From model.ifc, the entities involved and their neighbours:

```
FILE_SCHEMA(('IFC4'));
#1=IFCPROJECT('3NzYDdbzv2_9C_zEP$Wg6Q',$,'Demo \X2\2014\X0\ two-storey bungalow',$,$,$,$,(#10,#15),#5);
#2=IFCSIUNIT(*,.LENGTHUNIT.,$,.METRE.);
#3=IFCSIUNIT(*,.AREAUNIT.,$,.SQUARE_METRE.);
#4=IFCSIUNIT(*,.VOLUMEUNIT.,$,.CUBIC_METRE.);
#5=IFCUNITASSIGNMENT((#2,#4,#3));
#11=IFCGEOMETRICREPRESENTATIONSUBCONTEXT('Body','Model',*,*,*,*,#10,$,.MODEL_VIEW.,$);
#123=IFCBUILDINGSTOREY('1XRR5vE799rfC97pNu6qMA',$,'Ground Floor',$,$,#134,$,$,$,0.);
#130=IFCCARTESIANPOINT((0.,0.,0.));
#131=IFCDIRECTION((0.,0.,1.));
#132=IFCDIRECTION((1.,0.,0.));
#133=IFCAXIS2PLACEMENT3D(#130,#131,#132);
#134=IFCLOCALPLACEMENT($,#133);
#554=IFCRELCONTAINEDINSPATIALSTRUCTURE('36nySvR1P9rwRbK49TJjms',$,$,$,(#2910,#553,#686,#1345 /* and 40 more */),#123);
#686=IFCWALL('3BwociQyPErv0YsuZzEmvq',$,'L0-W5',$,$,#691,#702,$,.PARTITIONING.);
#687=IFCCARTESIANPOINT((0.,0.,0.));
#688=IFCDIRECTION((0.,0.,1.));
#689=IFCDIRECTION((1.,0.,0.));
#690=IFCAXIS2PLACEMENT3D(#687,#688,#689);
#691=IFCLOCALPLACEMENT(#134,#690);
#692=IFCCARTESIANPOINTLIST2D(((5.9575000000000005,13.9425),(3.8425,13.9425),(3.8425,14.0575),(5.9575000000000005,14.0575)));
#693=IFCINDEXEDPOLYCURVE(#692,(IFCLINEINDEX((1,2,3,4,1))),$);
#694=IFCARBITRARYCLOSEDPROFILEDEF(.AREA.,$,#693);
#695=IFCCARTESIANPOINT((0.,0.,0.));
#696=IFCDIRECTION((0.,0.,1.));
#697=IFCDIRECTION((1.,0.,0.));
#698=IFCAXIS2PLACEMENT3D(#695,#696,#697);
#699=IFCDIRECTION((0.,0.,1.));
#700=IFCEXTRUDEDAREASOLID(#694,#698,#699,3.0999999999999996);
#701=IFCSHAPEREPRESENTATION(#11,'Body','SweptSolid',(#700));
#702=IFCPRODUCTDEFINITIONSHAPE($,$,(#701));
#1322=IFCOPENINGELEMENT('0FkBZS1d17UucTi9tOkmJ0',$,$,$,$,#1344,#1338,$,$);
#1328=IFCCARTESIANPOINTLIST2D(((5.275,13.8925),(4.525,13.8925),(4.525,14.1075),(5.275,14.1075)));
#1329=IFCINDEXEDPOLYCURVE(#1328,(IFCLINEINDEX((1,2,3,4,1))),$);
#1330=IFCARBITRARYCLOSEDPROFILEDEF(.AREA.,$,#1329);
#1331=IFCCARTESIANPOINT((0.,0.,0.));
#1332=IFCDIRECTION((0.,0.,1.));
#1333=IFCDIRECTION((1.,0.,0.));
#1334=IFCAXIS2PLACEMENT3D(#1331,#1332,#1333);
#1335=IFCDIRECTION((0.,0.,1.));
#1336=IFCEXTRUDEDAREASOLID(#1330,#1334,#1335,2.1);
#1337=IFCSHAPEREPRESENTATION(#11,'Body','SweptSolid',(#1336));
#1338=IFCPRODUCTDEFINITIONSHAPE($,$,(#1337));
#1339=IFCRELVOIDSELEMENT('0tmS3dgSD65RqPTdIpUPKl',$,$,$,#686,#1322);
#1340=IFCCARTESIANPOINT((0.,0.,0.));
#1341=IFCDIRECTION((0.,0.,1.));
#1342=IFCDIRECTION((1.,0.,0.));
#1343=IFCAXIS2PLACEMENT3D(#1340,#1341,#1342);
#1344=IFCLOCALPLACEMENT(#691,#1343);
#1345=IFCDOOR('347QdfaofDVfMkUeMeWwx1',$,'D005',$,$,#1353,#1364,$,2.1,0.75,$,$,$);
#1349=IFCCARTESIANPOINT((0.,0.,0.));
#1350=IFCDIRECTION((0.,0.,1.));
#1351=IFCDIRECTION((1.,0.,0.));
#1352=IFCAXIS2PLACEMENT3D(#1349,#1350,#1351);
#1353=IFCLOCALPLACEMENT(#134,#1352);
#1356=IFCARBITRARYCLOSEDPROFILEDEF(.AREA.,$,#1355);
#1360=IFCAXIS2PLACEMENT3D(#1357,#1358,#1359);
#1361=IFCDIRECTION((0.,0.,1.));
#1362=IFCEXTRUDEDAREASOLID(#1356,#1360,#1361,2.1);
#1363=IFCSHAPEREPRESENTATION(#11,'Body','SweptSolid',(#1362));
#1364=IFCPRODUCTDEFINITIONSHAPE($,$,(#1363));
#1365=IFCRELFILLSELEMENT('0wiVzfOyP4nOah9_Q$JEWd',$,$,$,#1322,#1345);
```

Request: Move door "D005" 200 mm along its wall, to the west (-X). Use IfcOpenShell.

```python
import ifcopenshell
import ifcopenshell.api.geometry
import ifcopenshell.util.placement
import ifcopenshell.util.unit

model = ifcopenshell.open("model.ifc")
unit_scale = ifcopenshell.util.unit.calculate_unit_scale(model)

door = model.by_guid("347QdfaofDVfMkUeMeWwx1")
opening = door.FillsVoids[0].RelatingOpeningElement
wall = opening.VoidsElements[0].RelatingBuildingElement

wall_matrix = ifcopenshell.util.placement.get_local_placement(wall.ObjectPlacement)
shift = wall_matrix[:3, 0] * -0.2 / unit_scale
before = ifcopenshell.util.placement.get_local_placement(door.ObjectPlacement)[:3, 3].copy()

# The door is not placed relative to its opening, so move both.
for product in (opening, door):
    matrix = ifcopenshell.util.placement.get_local_placement(product.ObjectPlacement)
    matrix[:3, 3] += shift
    ifcopenshell.api.geometry.edit_object_placement(model, product=product, matrix=matrix, is_si=False)

after = ifcopenshell.util.placement.get_local_placement(door.ObjectPlacement)[:3, 3]
print("door moved by", (after - before).round(3) + 0.0)

model.write("model-out.ifc")
```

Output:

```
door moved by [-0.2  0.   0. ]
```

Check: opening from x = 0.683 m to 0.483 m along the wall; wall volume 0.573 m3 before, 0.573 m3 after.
